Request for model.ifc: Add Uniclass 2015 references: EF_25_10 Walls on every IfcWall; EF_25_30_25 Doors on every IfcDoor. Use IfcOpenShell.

First a look at what the model holds.

```python
import ifcopenshell

model = ifcopenshell.open("model.ifc")
print(model.schema)
print("classifications:", [c.Name for c in model.by_type("IfcClassification")])
for ifc_class in ("IfcDoor", "IfcRoof", "IfcStair", "IfcWall", "IfcWindow"):
    print(ifc_class, len(model.by_type(ifc_class)))
```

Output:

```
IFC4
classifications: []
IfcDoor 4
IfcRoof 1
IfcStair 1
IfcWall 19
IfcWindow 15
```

```python
import ifcopenshell
import ifcopenshell.api.classification

model = ifcopenshell.open("model.ifc")

system = ifcopenshell.api.classification.add_classification(model, classification="Uniclass 2015")

codes = {
    "IfcWall": ("EF_25_10", "Walls"),
    "IfcDoor": ("EF_25_30_25", "Doors"),
}
for ifc_class, (code, name) in codes.items():
    products = model.by_type(ifc_class)
    ifcopenshell.api.classification.add_reference(
        model, products=products, classification=system, identification=code, name=name
    )
    print(code, len(products))

model.write("model-out.ifc")
```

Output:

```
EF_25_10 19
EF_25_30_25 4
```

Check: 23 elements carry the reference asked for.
